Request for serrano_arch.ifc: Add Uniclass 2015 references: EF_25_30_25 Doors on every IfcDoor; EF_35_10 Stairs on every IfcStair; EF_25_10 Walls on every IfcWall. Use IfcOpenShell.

First a look at what the model holds.

```python
import ifcopenshell

model = ifcopenshell.open("serrano_arch.ifc")
print(model.schema)
print("classifications:", [c.Name for c in model.by_type("IfcClassification")])
for ifc_class in ("IfcDoor", "IfcRoof", "IfcStair", "IfcWall", "IfcWindow"):
    print(ifc_class, len(model.by_type(ifc_class)))
```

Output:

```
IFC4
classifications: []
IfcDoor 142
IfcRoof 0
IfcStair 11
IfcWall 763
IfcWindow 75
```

```python
import ifcopenshell
import ifcopenshell.api.classification

model = ifcopenshell.open("serrano_arch.ifc")

system = ifcopenshell.api.classification.add_classification(model, classification="Uniclass 2015")

codes = {
    "IfcDoor": ("EF_25_30_25", "Doors"),
    "IfcStair": ("EF_35_10", "Stairs"),
    "IfcWall": ("EF_25_10", "Walls"),
}
for ifc_class, (code, name) in codes.items():
    products = model.by_type(ifc_class)
    ifcopenshell.api.classification.add_reference(
        model, products=products, classification=system, identification=code, name=name
    )
    print(code, len(products))

model.write("serrano_arch_v2.ifc")
```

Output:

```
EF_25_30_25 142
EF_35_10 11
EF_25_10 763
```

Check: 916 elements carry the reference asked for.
